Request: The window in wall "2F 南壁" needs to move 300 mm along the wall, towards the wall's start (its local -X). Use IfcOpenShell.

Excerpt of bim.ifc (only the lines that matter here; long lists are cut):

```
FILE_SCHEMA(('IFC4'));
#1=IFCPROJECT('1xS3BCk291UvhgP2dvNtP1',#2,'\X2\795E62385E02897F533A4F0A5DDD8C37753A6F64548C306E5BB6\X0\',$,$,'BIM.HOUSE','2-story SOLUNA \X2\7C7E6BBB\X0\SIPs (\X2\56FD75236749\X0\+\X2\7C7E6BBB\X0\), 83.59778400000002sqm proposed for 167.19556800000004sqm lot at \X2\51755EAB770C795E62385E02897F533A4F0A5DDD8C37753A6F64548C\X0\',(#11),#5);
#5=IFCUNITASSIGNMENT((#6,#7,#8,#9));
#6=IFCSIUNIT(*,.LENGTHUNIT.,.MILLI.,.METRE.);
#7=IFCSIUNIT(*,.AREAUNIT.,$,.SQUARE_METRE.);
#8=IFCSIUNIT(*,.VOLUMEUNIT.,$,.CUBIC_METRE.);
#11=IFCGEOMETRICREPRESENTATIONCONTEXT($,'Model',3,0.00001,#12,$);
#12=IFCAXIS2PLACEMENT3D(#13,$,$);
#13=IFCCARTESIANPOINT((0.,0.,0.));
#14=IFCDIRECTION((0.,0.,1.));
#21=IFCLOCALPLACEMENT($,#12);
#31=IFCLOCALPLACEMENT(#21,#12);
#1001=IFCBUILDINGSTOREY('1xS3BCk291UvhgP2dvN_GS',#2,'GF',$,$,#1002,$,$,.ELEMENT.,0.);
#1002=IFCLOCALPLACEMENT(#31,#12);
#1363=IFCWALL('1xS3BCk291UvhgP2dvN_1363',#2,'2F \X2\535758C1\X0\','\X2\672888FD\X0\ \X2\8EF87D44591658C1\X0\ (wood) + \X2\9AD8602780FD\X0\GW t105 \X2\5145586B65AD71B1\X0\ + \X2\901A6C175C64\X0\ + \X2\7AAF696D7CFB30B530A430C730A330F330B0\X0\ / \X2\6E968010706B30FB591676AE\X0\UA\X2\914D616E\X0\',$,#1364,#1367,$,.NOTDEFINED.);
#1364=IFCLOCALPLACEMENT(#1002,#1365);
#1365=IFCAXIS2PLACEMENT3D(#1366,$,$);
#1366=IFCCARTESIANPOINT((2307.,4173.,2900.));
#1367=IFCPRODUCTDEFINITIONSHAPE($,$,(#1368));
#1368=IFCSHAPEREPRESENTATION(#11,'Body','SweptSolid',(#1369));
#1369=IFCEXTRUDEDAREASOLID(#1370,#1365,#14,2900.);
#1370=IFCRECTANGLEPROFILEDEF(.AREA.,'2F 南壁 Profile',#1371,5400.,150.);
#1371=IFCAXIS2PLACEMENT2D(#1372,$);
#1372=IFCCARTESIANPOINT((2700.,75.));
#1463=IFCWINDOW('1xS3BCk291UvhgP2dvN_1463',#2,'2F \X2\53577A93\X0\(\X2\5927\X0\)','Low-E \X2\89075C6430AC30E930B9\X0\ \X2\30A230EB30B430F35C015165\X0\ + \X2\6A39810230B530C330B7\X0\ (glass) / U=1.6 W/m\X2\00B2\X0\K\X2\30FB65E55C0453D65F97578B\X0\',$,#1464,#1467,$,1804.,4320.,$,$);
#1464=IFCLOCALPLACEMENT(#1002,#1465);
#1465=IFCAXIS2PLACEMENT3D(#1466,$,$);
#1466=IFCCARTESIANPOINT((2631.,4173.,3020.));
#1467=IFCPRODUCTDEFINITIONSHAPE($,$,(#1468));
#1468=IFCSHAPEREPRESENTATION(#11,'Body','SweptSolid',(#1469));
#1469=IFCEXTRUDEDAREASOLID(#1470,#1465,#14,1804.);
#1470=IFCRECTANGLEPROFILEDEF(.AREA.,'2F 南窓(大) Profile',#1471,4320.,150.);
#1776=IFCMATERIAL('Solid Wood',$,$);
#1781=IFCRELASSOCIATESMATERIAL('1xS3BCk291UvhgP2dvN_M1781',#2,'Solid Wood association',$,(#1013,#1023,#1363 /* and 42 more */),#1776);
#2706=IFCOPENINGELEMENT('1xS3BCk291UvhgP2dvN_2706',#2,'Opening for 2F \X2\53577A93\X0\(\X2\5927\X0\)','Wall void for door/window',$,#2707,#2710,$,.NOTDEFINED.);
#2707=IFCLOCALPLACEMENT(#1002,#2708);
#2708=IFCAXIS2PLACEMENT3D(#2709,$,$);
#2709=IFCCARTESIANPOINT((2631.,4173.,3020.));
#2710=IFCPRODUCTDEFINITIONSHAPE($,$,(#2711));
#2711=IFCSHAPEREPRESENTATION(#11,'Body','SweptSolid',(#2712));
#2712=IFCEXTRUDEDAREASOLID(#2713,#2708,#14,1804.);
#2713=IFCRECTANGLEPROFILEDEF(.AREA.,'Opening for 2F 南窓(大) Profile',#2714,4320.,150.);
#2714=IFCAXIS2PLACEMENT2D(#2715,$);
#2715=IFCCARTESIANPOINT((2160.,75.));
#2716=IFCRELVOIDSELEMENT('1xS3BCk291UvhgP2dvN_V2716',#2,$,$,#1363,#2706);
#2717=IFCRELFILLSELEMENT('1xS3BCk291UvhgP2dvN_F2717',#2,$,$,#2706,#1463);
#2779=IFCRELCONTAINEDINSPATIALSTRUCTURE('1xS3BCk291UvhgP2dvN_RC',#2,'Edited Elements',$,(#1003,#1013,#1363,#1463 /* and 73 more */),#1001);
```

```python
import ifcopenshell
import ifcopenshell.api.geometry
import ifcopenshell.util.placement

model = ifcopenshell.open("bim.ifc")

window = model.by_guid("1xS3BCk291UvhgP2dvN_1463")
opening = window.FillsVoids[0].RelatingOpeningElement
wall = opening.VoidsElements[0].RelatingBuildingElement

wall_matrix = ifcopenshell.util.placement.get_local_placement(wall.ObjectPlacement)
shift = wall_matrix[:3, 0] * -300.0
before = ifcopenshell.util.placement.get_local_placement(window.ObjectPlacement)[:3, 3].copy()

# The window is not placed relative to its opening, so move both.
for product in (opening, window):
    matrix = ifcopenshell.util.placement.get_local_placement(product.ObjectPlacement)
    matrix[:3, 3] += shift
    ifcopenshell.api.geometry.edit_object_placement(model, product=product, matrix=matrix, is_si=False)

after = ifcopenshell.util.placement.get_local_placement(window.ObjectPlacement)[:3, 3]
print("window moved by", (after - before).round(3) + 0.0)

model.write("bim_updated.ifc")
```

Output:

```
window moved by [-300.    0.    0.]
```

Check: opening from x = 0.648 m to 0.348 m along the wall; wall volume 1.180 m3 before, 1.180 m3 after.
